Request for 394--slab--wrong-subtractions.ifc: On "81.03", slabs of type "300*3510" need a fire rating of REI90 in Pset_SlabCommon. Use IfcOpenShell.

First a look at what the model holds.

```python
import ifcopenshell
import ifcopenshell.util.element

model = ifcopenshell.open("394--slab--wrong-subtractions.ifc")
print(model.schema)
storey = next(s for s in model.by_type("IfcBuildingStorey") if s.Name == "81.03")
slabs = [e for e in ifcopenshell.util.element.get_decomposition(storey) if e.is_a("IfcSlab")]
seen = {}
for e in slabs:
    element_type = ifcopenshell.util.element.get_type(e)
    key = (element_type.Name if element_type != e and element_type else None, ifcopenshell.util.element.get_pset(e, "Pset_SlabCommon", "FireRating"))
    seen[key] = seen.get(key, 0) + 1
for (name, value), count in sorted(seen.items(), key=str):
    print(count, "x", name, "|", value)
```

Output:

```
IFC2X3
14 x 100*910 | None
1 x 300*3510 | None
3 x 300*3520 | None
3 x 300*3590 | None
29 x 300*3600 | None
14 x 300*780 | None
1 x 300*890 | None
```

```python
import ifcopenshell
import ifcopenshell.api.pset
import ifcopenshell.util.element

model = ifcopenshell.open("394--slab--wrong-subtractions.ifc")

storey = next(s for s in model.by_type("IfcBuildingStorey") if s.Name == "81.03")
slabs = [e for e in ifcopenshell.util.element.get_decomposition(storey) if e.is_a("IfcSlab")]

count = 0
for e in slabs:
    element_type = ifcopenshell.util.element.get_type(e)
    if element_type in (None, e) or element_type.Name != "300*3510":
        continue
    # add_pset returns the element's existing set when there is one.
    pset = ifcopenshell.api.pset.add_pset(model, product=e, name="Pset_SlabCommon")
    ifcopenshell.api.pset.edit_pset(model, pset=pset, properties={"FireRating": "REI90"})
    count += 1

print(count, "slabs updated")

model.write("394--slab--wrong-subtractions-out.ifc")
```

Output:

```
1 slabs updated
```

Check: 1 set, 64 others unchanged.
